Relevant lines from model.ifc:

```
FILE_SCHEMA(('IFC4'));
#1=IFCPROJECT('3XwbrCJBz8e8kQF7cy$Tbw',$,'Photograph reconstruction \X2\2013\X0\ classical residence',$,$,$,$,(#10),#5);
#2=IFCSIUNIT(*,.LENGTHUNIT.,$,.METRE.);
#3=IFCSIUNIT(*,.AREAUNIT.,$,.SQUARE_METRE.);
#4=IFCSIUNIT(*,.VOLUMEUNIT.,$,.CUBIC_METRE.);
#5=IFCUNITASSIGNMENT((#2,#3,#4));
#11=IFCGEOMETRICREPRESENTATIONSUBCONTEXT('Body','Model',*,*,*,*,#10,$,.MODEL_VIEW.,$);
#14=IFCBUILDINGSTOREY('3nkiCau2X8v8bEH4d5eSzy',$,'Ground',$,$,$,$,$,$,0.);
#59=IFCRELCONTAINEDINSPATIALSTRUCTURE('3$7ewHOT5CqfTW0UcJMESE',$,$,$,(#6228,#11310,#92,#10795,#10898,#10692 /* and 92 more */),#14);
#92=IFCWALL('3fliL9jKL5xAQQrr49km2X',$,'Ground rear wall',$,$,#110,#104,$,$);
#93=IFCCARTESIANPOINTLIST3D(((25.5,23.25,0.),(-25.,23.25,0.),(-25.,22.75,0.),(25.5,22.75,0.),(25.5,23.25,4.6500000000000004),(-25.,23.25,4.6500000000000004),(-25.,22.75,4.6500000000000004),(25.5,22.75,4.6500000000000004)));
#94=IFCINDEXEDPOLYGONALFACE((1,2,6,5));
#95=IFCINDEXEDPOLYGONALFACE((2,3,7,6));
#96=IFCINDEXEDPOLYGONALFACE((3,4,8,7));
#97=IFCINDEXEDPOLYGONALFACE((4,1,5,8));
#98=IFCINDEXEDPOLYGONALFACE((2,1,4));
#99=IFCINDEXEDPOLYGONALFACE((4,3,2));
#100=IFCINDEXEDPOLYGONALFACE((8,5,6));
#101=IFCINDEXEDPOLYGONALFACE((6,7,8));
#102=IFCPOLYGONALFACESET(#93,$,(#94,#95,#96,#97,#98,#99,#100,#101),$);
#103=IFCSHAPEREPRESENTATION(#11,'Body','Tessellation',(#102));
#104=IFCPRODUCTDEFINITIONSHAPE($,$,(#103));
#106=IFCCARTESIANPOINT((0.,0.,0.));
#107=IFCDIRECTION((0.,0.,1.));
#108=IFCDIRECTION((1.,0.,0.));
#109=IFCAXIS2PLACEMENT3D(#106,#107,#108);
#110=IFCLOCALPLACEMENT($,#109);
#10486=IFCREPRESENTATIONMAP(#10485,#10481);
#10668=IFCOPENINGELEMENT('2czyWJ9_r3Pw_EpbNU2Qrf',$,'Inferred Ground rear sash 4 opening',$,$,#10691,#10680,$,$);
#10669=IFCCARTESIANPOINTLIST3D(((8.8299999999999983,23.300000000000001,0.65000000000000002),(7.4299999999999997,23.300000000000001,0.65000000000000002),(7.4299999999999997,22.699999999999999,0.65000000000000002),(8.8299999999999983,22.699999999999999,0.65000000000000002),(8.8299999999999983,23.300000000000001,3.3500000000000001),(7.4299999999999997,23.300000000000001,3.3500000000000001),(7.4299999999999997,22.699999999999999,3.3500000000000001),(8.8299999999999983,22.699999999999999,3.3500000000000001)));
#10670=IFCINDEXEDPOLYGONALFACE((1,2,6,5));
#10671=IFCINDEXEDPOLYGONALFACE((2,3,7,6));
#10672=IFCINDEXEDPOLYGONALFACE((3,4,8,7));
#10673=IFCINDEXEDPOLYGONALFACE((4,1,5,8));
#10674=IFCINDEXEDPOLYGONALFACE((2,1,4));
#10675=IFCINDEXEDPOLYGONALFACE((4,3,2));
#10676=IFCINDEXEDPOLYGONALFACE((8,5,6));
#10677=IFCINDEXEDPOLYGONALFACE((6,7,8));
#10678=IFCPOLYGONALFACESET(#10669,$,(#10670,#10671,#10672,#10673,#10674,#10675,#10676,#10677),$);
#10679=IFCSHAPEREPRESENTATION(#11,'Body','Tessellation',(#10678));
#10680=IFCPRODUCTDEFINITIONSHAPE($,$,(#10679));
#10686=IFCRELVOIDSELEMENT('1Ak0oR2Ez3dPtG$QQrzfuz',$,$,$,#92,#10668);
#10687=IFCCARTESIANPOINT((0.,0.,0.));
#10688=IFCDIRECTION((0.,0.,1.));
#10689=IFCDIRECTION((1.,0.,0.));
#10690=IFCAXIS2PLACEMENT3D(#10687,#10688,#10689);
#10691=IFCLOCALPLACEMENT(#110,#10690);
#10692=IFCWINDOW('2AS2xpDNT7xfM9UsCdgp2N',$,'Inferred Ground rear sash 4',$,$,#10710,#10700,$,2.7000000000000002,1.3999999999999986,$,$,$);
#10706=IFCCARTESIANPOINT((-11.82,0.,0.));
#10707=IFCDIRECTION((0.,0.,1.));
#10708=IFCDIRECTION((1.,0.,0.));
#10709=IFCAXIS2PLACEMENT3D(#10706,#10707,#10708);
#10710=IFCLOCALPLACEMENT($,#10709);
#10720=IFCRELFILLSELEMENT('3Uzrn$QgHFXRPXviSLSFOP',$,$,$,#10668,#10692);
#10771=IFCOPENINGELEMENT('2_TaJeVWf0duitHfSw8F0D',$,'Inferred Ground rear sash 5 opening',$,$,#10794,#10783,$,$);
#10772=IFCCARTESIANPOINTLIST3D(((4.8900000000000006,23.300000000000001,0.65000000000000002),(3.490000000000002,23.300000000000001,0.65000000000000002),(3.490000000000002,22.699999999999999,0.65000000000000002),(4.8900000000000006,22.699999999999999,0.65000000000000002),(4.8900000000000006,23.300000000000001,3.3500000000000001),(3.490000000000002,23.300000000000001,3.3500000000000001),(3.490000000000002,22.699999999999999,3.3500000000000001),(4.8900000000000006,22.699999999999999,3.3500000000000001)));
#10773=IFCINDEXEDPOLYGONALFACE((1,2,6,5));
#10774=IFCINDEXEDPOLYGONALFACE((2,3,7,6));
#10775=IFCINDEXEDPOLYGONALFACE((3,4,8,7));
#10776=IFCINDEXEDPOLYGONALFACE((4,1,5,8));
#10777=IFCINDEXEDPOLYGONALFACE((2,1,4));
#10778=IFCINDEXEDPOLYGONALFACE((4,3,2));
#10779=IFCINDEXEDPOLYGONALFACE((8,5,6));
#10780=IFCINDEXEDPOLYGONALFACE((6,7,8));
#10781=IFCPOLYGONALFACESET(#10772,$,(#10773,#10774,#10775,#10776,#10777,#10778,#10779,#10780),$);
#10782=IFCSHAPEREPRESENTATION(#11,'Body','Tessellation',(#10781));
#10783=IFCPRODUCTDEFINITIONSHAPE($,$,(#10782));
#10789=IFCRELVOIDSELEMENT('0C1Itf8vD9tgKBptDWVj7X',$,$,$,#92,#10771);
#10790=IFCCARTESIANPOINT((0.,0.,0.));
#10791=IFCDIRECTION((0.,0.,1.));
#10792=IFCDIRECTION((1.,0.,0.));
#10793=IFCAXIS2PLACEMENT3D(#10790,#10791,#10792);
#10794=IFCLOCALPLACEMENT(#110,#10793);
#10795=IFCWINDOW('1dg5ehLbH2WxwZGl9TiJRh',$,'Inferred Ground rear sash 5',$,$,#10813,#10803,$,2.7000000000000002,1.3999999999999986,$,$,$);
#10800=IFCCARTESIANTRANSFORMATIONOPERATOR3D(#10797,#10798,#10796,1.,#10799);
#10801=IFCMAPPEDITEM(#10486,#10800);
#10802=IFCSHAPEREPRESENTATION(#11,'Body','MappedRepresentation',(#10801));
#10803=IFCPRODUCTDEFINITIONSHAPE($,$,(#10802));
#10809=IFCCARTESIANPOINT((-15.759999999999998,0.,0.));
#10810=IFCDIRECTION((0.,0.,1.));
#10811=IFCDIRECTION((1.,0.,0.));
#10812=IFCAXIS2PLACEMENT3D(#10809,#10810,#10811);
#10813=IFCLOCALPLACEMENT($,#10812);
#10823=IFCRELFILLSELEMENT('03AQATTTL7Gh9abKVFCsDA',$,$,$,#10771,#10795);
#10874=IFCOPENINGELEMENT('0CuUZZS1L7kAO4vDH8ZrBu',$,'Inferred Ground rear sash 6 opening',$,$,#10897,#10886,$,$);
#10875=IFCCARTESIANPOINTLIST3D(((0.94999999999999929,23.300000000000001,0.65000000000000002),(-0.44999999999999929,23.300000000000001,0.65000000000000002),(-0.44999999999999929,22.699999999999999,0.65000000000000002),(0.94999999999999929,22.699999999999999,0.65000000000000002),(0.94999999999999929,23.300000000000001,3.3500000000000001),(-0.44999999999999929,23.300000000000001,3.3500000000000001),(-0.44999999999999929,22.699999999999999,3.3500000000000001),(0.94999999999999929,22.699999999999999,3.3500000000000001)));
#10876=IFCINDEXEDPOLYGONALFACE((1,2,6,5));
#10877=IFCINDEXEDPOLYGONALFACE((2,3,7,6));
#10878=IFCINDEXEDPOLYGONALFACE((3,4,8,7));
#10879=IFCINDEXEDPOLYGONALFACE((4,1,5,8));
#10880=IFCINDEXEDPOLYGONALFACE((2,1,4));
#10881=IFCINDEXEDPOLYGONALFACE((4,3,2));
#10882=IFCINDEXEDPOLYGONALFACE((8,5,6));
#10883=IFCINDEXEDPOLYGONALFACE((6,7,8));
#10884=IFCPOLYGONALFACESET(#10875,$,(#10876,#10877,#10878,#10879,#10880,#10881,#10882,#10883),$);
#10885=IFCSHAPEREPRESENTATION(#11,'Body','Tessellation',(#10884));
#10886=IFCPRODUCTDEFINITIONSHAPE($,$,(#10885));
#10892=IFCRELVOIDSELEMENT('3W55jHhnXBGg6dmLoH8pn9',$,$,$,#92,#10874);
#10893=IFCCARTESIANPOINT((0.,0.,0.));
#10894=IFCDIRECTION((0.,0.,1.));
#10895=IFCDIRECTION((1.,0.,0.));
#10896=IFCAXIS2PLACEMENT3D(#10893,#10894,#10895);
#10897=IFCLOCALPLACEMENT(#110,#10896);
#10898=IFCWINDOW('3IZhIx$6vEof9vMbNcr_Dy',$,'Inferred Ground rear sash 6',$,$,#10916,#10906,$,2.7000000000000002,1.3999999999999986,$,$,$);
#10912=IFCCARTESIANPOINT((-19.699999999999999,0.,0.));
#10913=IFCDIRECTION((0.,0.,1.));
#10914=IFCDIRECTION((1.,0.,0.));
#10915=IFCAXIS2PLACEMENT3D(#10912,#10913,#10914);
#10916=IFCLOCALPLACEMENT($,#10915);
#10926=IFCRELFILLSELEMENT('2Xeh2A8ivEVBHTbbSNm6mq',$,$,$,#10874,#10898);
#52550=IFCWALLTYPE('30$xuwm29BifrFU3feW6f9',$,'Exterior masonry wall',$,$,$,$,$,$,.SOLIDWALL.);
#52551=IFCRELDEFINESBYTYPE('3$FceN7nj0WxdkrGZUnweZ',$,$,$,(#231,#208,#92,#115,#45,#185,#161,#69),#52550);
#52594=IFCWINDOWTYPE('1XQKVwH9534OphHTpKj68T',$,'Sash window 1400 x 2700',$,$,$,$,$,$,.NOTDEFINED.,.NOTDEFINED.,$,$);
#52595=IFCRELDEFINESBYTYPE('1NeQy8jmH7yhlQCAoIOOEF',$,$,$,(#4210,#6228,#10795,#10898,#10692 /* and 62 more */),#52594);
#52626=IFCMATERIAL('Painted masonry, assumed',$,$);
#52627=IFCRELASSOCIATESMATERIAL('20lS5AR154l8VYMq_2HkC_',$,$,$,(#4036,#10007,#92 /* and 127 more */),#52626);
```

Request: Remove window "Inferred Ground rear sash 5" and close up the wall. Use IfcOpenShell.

```python
import ifcopenshell
import ifcopenshell.api.feature
import ifcopenshell.api.root
import ifcopenshell.geom
import ifcopenshell.util.shape

model = ifcopenshell.open("model.ifc")
settings = ifcopenshell.geom.settings()


def volume(element):
    """Net volume in cubic metres, openings subtracted."""
    shape = ifcopenshell.geom.create_shape(settings, element)
    return ifcopenshell.util.shape.get_volume(shape.geometry)


window = model.by_guid("1dg5ehLbH2WxwZGl9TiJRh")
opening = window.FillsVoids[0].RelatingOpeningElement
wall = opening.VoidsElements[0].RelatingBuildingElement
before = volume(wall)

ifcopenshell.api.root.remove_product(model, product=window)
ifcopenshell.api.feature.remove_feature(model, feature=opening)

after = volume(wall)

print(f"wall volume {before:.3f} -> {after:.3f} m3")

model.write("model_updated.ifc")
```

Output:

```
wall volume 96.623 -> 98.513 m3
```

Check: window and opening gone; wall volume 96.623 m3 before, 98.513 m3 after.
